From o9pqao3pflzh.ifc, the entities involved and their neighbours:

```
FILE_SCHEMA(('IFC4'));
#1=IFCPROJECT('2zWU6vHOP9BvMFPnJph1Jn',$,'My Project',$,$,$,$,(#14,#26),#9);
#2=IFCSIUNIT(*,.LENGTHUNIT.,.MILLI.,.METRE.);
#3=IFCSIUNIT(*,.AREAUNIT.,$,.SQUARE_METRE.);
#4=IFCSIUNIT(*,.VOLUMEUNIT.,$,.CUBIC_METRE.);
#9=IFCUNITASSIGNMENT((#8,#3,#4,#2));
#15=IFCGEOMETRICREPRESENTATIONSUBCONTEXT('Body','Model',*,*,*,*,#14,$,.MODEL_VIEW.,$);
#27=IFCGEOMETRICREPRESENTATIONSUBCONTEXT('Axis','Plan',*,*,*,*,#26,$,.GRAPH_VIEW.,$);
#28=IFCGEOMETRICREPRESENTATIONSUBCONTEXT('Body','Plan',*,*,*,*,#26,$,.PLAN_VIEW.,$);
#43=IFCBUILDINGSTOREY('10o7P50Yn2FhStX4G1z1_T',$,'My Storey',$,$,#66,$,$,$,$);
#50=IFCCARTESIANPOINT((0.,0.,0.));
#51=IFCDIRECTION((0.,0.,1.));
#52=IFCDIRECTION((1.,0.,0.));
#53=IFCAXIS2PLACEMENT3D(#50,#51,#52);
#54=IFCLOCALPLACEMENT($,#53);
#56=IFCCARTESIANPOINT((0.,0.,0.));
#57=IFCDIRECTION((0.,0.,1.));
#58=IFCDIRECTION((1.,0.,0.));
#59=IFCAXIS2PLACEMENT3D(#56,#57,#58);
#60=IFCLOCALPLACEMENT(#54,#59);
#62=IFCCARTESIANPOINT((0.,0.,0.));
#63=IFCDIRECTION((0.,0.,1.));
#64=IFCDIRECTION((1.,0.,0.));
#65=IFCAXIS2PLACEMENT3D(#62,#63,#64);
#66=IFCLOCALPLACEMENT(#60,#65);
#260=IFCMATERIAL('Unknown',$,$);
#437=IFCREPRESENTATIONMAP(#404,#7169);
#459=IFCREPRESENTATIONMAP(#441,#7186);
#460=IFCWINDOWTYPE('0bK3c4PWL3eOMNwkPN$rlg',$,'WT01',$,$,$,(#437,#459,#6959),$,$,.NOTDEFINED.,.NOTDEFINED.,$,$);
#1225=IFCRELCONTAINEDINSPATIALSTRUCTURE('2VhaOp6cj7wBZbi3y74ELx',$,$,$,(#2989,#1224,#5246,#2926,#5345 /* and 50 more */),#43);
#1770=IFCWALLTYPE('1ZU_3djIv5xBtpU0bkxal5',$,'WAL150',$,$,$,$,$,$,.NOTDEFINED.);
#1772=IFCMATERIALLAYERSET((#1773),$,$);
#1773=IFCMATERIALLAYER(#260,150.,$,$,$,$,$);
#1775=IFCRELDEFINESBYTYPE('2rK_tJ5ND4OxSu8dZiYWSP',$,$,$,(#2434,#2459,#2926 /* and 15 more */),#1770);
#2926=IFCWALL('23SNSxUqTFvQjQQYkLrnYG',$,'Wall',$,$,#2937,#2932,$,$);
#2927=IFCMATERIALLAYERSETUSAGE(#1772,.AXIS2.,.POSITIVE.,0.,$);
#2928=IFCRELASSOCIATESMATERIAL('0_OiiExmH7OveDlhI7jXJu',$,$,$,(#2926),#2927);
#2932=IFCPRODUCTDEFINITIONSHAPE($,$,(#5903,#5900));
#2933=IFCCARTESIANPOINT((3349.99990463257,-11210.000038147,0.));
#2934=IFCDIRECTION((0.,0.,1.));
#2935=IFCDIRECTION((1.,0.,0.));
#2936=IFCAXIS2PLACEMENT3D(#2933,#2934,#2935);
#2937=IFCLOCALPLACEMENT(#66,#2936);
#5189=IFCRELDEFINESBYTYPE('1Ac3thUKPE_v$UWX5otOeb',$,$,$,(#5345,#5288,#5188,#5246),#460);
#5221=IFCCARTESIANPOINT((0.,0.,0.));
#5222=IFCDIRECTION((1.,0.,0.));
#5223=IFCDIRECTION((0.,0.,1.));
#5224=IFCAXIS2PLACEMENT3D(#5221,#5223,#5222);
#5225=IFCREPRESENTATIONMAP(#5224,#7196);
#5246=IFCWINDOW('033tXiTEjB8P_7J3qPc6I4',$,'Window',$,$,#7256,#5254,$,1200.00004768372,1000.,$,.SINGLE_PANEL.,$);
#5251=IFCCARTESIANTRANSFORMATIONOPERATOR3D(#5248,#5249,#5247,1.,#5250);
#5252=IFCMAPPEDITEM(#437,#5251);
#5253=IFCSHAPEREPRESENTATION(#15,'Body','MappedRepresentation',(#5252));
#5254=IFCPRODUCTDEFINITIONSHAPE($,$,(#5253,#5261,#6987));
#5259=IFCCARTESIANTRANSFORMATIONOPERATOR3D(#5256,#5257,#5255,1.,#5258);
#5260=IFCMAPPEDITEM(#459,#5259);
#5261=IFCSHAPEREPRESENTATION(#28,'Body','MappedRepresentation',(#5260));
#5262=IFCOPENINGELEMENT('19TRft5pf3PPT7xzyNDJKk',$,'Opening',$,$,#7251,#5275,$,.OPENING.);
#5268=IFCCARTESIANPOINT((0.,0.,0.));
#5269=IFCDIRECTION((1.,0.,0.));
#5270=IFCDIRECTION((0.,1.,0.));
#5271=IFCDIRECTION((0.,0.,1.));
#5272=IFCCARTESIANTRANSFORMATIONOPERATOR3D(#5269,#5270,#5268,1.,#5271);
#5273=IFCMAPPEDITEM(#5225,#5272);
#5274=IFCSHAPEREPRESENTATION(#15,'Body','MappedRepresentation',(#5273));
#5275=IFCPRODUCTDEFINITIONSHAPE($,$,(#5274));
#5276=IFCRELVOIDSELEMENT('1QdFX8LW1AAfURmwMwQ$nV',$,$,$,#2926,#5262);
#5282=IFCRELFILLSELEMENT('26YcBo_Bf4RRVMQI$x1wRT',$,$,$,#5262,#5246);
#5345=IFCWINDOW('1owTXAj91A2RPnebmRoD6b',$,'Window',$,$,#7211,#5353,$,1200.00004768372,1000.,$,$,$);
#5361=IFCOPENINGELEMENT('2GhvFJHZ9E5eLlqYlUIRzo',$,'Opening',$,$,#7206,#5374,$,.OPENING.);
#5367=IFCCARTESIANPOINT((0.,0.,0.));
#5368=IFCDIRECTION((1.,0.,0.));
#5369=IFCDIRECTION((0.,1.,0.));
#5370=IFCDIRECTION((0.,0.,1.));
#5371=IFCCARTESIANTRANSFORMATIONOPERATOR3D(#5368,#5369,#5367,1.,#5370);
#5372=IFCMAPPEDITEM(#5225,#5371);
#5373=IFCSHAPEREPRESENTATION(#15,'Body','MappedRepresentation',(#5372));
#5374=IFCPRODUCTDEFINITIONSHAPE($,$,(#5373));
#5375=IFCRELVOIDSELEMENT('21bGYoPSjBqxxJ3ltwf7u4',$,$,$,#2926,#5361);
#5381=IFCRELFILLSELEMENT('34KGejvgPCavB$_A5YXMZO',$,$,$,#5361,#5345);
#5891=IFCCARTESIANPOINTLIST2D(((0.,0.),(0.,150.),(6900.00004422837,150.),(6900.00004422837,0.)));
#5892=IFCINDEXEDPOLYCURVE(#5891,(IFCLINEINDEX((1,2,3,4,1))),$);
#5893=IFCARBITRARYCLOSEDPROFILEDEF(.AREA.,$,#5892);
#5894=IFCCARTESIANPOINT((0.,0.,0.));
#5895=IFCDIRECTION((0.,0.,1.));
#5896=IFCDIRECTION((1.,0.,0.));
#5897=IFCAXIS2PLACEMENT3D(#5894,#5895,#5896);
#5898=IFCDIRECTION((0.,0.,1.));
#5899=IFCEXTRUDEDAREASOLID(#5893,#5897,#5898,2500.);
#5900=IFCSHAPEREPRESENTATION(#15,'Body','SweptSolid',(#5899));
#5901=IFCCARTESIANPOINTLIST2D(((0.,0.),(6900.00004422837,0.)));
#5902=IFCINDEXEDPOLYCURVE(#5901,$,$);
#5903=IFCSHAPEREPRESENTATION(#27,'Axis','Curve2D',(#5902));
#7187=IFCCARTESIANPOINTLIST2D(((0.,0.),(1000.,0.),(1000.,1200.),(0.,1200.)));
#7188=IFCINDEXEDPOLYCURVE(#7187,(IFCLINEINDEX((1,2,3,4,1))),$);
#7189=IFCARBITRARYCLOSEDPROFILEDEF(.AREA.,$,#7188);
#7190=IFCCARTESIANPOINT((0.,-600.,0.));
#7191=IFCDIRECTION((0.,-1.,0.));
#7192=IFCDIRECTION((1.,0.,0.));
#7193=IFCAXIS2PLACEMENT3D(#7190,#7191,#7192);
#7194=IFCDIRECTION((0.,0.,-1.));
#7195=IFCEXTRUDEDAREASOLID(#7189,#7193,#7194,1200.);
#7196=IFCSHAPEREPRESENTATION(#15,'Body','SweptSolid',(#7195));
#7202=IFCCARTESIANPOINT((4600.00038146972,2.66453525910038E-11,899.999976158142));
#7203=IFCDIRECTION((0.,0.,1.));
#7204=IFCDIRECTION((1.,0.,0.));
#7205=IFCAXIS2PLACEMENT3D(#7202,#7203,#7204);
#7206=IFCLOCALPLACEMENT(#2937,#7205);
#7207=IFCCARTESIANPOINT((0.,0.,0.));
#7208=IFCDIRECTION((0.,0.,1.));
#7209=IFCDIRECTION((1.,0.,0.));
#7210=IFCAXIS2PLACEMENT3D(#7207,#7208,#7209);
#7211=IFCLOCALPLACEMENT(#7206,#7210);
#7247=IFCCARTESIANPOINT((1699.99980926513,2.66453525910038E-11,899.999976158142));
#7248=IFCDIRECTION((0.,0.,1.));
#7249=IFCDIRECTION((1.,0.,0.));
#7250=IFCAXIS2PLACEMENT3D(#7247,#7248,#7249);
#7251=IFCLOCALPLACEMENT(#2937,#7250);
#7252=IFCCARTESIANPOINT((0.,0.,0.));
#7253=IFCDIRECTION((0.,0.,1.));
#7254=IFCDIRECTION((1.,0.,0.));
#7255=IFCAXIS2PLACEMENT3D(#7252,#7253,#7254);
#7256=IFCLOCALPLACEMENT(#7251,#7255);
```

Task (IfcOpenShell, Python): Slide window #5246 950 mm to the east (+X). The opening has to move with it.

```python
import ifcopenshell
import ifcopenshell.api.geometry
import ifcopenshell.util.placement
import ifcopenshell.util.unit

model = ifcopenshell.open("o9pqao3pflzh.ifc")
unit_scale = ifcopenshell.util.unit.calculate_unit_scale(model)

window = model.by_guid("033tXiTEjB8P_7J3qPc6I4")
opening = window.FillsVoids[0].RelatingOpeningElement
wall = opening.VoidsElements[0].RelatingBuildingElement

wall_matrix = ifcopenshell.util.placement.get_local_placement(wall.ObjectPlacement)
shift = wall_matrix[:3, 0] * 0.95 / unit_scale
before = ifcopenshell.util.placement.get_local_placement(window.ObjectPlacement)[:3, 3].copy()

# The window is placed relative to its opening, so it follows when the opening moves.
matrix = ifcopenshell.util.placement.get_local_placement(opening.ObjectPlacement)
matrix[:3, 3] += shift
ifcopenshell.api.geometry.edit_object_placement(
    model, product=opening, matrix=matrix, is_si=False, should_transform_children=True
)

after = ifcopenshell.util.placement.get_local_placement(window.ObjectPlacement)[:3, 3]
print("window moved by", (after - before).round(3) + 0.0)

model.write("o9pqao3pflzh-out.ifc")
```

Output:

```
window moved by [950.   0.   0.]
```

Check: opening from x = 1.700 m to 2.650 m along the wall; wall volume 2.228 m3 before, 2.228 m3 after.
